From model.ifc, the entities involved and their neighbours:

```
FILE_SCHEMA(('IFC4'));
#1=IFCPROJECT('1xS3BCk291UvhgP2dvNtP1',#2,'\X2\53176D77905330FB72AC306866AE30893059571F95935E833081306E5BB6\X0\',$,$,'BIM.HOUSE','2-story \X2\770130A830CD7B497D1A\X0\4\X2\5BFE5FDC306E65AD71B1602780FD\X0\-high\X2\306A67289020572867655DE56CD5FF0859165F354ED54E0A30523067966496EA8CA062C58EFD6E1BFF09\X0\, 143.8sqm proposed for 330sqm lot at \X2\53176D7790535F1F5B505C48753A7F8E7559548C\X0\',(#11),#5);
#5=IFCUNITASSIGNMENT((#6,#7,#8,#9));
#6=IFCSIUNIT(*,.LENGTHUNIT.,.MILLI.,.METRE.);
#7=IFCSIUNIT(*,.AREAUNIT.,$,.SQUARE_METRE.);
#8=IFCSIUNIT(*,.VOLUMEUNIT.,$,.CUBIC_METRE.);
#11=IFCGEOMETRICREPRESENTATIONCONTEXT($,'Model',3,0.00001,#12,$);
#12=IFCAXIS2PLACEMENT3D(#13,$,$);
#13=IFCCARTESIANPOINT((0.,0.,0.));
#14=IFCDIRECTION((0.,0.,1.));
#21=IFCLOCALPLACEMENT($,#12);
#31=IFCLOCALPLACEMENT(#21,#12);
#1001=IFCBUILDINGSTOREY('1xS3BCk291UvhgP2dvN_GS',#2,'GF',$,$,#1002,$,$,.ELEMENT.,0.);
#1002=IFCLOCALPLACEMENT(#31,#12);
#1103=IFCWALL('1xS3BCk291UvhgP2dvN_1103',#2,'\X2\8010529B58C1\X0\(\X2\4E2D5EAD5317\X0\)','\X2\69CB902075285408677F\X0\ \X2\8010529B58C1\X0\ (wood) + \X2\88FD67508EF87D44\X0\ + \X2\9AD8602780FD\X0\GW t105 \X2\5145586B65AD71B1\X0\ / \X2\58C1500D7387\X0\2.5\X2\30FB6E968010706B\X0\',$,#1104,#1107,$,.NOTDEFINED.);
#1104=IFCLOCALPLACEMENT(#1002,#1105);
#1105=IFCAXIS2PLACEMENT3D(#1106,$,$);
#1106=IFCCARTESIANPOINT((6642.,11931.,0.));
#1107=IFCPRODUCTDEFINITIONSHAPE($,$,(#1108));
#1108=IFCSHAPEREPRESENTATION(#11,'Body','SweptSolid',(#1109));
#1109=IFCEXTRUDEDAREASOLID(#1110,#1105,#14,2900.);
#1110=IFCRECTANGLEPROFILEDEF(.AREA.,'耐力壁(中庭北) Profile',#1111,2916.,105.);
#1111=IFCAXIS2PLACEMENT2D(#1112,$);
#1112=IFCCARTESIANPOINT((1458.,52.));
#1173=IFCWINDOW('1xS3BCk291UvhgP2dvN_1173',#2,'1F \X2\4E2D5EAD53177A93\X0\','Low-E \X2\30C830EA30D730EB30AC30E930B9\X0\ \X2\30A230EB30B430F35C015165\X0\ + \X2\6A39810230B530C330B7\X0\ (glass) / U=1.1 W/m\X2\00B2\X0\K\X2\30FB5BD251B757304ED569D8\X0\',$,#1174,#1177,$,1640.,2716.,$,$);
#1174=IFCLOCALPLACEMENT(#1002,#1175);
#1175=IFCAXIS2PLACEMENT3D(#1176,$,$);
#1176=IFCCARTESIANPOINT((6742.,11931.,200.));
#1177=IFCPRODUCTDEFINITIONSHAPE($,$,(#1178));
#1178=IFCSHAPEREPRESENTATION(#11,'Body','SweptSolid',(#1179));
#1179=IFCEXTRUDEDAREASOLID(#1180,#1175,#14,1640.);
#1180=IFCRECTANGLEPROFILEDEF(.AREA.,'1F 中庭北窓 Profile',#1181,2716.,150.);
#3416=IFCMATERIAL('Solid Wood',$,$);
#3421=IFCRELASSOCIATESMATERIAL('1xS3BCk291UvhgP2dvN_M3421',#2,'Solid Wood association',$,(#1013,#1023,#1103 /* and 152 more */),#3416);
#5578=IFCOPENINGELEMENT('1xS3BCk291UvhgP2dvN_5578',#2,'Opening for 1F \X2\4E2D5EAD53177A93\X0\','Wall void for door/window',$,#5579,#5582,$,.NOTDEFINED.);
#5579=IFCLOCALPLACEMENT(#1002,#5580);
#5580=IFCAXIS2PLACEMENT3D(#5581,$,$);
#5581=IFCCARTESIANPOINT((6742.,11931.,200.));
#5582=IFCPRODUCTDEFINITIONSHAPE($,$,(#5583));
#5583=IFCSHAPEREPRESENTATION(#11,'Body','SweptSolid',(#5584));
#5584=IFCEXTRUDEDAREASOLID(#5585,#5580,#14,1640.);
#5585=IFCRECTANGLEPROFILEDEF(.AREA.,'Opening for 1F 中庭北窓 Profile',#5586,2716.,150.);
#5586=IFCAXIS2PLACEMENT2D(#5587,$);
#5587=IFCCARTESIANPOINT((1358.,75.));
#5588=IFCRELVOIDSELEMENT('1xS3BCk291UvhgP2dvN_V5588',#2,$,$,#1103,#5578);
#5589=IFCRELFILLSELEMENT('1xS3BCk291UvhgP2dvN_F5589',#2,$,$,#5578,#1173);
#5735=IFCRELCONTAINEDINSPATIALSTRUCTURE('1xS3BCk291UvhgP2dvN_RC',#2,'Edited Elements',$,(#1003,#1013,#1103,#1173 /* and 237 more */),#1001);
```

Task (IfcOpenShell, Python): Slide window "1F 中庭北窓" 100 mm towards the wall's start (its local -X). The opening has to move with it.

```python
import ifcopenshell
import ifcopenshell.api.geometry
import ifcopenshell.util.placement
import ifcopenshell.util.unit

model = ifcopenshell.open("model.ifc")
unit_scale = ifcopenshell.util.unit.calculate_unit_scale(model)

window = model.by_guid("1xS3BCk291UvhgP2dvN_1173")
opening = window.FillsVoids[0].RelatingOpeningElement
wall = opening.VoidsElements[0].RelatingBuildingElement

wall_matrix = ifcopenshell.util.placement.get_local_placement(wall.ObjectPlacement)
shift = wall_matrix[:3, 0] * -0.1 / unit_scale
before = ifcopenshell.util.placement.get_local_placement(window.ObjectPlacement)[:3, 3].copy()

# The window is not placed relative to its opening, so move both.
for product in (opening, window):
    matrix = ifcopenshell.util.placement.get_local_placement(product.ObjectPlacement)
    matrix[:3, 3] += shift
    ifcopenshell.api.geometry.edit_object_placement(model, product=product, matrix=matrix, is_si=False)

after = ifcopenshell.util.placement.get_local_placement(window.ObjectPlacement)[:3, 3]
print("window moved by", (after - before).round(3) + 0.0)

model.write("model_v2.ifc")
```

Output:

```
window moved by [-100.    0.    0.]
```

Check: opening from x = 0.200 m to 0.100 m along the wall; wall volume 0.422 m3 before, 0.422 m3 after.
